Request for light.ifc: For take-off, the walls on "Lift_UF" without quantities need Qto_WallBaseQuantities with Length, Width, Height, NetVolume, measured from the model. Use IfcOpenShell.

First a look at what the model holds.

```python
import ifcopenshell
import ifcopenshell.util.element
import ifcopenshell.util.unit

model = ifcopenshell.open("light.ifc")
print(model.schema)
for unit_type in ("LENGTHUNIT", "AREAUNIT", "VOLUMEUNIT"):
    print(unit_type, ifcopenshell.util.unit.calculate_unit_scale(model, unit_type))
storey = next(s for s in model.by_type("IfcBuildingStorey") if s.Name == "Lift_UF")
walls = [e for e in ifcopenshell.util.element.get_decomposition(storey) if e.is_a("IfcWall")]
for e in sorted(walls, key=lambda e: e.id()):
    print(e.id(), e.is_a(), e.Name, list(ifcopenshell.util.element.get_psets(e, qtos_only=True)), sep=" | ")
```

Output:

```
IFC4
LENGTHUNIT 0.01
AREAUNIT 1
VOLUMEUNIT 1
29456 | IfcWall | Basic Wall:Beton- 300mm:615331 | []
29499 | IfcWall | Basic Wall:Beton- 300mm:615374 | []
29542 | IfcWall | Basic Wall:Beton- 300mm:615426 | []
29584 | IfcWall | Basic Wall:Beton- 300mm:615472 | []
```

```python
import ifcopenshell
import ifcopenshell.api.pset
import ifcopenshell.geom
import ifcopenshell.util.element
import ifcopenshell.util.shape
import ifcopenshell.util.unit

model = ifcopenshell.open("light.ifc")
unit_scale = ifcopenshell.util.unit.calculate_unit_scale(model)
volume_scale = ifcopenshell.util.unit.calculate_unit_scale(model, "VOLUMEUNIT")
settings = ifcopenshell.geom.settings()

storey = next(s for s in model.by_type("IfcBuildingStorey") if s.Name == "Lift_UF")
walls = [e for e in ifcopenshell.util.element.get_decomposition(storey) if e.is_a("IfcWall")]

for e in sorted(walls, key=lambda e: e.id()):
    if ifcopenshell.util.element.get_psets(e, qtos_only=True, should_inherit=False):
        continue
    # Geometry comes back in metres, in the element's own axes.
    shape = ifcopenshell.geom.create_shape(settings, e)
    values = {
        "Length": ifcopenshell.util.shape.get_x(shape.geometry) / unit_scale,
        "Width": ifcopenshell.util.shape.get_y(shape.geometry) / unit_scale,
        "Height": ifcopenshell.util.shape.get_z(shape.geometry) / unit_scale,
        "NetVolume": ifcopenshell.util.shape.get_volume(shape.geometry) / volume_scale,
    }
    qto = ifcopenshell.api.pset.add_qto(model, product=e, name="Qto_WallBaseQuantities")
    ifcopenshell.api.pset.edit_qto(model, qto=qto, properties=values)
    print(e.id(), {k: round(v, 3) for k, v in values.items()})

model.write("light_rev.ifc")
```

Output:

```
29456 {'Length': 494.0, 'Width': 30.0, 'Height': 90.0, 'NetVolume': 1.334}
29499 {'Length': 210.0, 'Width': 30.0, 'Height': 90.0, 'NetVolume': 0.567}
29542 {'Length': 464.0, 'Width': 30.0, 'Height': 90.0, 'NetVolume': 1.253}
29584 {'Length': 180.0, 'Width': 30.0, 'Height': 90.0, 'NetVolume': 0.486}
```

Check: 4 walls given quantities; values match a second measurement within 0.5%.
